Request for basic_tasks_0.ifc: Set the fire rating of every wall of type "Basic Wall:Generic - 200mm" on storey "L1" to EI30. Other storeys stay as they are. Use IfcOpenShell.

First a look at what the model holds.

```python
import ifcopenshell
import ifcopenshell.util.element

model = ifcopenshell.open("basic_tasks_0.ifc")
print(model.schema)
storey = next(s for s in model.by_type("IfcBuildingStorey") if s.Name == "L1")
walls = [e for e in ifcopenshell.util.element.get_decomposition(storey) if e.is_a("IfcWall")]
seen = {}
for e in walls:
    element_type = ifcopenshell.util.element.get_type(e)
    key = (element_type.Name if element_type != e and element_type else None, ifcopenshell.util.element.get_pset(e, "Pset_WallCommon", "FireRating"))
    seen[key] = seen.get(key, 0) + 1
for (name, value), count in sorted(seen.items(), key=str):
    print(count, "x", name, "|", value)
```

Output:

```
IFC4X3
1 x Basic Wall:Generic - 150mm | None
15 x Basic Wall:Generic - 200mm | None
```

```python
import ifcopenshell
import ifcopenshell.api.pset
import ifcopenshell.util.element

model = ifcopenshell.open("basic_tasks_0.ifc")

storey = next(s for s in model.by_type("IfcBuildingStorey") if s.Name == "L1")
walls = [e for e in ifcopenshell.util.element.get_decomposition(storey) if e.is_a("IfcWall")]

count = 0
for e in walls:
    element_type = ifcopenshell.util.element.get_type(e)
    if element_type in (None, e) or element_type.Name != "Basic Wall:Generic - 200mm":
        continue
    # add_pset returns the element's existing set when there is one.
    pset = ifcopenshell.api.pset.add_pset(model, product=e, name="Pset_WallCommon")
    ifcopenshell.api.pset.edit_pset(model, pset=pset, properties={"FireRating": "EI30"})
    count += 1

print(count, "walls updated")

model.write("basic_tasks_0_rev.ifc")
```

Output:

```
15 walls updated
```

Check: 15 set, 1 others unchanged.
